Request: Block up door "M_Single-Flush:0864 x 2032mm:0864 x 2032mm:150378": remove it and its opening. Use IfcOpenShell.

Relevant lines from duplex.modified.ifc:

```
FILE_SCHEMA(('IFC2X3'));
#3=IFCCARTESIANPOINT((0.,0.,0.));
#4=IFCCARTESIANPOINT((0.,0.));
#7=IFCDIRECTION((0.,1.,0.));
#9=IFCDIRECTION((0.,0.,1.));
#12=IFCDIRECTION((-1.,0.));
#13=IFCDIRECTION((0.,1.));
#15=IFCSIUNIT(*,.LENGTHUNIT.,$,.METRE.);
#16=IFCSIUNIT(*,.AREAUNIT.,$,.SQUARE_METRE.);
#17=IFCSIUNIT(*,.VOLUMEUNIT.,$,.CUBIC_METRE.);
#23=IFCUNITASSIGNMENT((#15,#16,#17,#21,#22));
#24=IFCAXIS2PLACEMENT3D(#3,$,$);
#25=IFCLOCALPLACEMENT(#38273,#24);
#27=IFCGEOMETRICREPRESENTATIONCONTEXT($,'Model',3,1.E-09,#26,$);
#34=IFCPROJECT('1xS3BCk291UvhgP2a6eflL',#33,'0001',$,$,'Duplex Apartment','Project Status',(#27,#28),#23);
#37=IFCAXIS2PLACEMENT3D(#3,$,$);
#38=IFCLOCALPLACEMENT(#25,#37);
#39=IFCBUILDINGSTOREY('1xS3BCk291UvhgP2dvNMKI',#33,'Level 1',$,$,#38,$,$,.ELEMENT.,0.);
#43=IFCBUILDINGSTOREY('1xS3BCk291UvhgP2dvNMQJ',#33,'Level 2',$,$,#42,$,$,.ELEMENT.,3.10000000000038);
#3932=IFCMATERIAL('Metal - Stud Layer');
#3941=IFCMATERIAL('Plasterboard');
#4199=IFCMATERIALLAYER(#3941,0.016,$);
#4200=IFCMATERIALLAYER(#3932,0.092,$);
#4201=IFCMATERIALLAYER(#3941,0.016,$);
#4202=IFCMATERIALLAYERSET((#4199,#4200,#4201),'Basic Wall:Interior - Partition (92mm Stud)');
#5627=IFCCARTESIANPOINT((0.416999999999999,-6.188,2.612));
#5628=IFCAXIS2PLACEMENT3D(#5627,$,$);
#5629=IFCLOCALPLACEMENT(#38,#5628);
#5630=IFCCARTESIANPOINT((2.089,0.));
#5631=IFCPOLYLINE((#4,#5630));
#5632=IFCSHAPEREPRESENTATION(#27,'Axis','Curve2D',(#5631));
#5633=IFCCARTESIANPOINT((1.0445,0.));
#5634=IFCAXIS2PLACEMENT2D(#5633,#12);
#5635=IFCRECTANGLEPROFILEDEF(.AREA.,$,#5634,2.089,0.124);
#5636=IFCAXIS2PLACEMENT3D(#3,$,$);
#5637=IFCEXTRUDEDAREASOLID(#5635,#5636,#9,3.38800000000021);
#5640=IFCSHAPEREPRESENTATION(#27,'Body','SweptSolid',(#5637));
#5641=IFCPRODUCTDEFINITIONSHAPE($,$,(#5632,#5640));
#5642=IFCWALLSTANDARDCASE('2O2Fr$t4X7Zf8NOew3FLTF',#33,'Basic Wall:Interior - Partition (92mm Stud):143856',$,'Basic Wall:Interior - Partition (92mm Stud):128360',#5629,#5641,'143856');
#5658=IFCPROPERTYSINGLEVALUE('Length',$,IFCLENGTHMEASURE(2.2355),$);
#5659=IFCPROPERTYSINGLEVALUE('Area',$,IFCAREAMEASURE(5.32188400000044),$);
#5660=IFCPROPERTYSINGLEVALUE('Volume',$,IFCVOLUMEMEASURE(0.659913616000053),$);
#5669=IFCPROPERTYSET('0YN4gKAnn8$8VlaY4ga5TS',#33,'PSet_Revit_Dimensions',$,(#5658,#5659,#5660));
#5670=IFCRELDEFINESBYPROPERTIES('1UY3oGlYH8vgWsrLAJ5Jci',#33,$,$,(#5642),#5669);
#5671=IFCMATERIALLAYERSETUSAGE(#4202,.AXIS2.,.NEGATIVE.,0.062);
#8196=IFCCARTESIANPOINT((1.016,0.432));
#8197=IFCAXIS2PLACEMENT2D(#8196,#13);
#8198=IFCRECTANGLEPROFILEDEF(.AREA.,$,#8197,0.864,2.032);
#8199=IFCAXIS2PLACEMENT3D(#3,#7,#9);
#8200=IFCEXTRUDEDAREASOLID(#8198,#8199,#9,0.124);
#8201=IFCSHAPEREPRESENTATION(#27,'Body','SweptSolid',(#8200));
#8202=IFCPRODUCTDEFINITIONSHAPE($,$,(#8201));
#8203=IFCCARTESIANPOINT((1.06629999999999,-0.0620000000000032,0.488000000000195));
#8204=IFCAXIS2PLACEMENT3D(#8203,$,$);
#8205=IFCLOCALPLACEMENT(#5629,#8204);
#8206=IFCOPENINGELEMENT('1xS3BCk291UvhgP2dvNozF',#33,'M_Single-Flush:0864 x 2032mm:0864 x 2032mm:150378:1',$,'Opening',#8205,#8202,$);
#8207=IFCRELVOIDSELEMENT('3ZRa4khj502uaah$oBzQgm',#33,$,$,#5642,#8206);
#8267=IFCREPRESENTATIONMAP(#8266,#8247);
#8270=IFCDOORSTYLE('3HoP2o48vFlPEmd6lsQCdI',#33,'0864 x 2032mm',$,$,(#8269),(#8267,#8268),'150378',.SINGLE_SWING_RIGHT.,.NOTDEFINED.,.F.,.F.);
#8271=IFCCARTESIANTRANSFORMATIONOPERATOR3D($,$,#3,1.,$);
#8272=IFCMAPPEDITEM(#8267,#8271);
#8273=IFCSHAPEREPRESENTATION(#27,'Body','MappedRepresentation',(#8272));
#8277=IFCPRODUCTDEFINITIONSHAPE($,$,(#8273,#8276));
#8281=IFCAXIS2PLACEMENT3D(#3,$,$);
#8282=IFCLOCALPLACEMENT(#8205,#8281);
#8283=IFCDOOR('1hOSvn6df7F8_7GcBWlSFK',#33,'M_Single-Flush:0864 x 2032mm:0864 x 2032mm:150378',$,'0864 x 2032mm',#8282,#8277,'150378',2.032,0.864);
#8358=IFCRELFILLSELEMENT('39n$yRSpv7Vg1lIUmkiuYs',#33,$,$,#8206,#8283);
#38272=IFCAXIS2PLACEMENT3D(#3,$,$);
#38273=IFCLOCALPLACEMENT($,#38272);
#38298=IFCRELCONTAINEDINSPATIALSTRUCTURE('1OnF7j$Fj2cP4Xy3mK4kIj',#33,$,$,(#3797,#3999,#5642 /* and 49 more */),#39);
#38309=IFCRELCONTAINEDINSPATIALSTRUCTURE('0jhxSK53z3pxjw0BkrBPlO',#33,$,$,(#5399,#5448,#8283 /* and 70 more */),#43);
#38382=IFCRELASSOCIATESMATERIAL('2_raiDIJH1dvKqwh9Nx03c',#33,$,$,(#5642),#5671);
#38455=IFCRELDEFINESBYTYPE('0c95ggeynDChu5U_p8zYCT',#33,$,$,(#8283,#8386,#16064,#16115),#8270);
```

```python
import ifcopenshell
import ifcopenshell.api.feature
import ifcopenshell.api.pset
import ifcopenshell.api.root
import ifcopenshell.geom
import ifcopenshell.util.element
import ifcopenshell.util.shape
import ifcopenshell.util.unit

model = ifcopenshell.open("duplex.modified.ifc")
area_scale = ifcopenshell.util.unit.calculate_unit_scale(model, "AREAUNIT")
volume_scale = ifcopenshell.util.unit.calculate_unit_scale(model, "VOLUMEUNIT")
settings = ifcopenshell.geom.settings()


def volume(element):
    """Net volume in cubic metres, openings subtracted."""
    shape = ifcopenshell.geom.create_shape(settings, element)
    return ifcopenshell.util.shape.get_volume(shape.geometry)


door = model.by_guid("1hOSvn6df7F8_7GcBWlSFK")
opening = door.FillsVoids[0].RelatingOpeningElement
wall = opening.VoidsElements[0].RelatingBuildingElement
before = volume(wall)

ifcopenshell.api.root.remove_product(model, product=door)
ifcopenshell.api.feature.remove_feature(model, feature=opening)

after = volume(wall)
thickness = 0.124  # wall thickness in metres

# Update the wall's stored quantities.
pset = model.by_id(ifcopenshell.util.element.get_pset(wall, "PSet_Revit_Dimensions", should_inherit=False)["id"])
ifcopenshell.api.pset.edit_pset(model, pset=pset, properties={
    "Area": model.create_entity("IfcAreaMeasure", after / thickness / area_scale),
    "Volume": model.create_entity("IfcVolumeMeasure", after / volume_scale),
})

print(f"wall volume {before:.3f} -> {after:.3f} m3")

model.write("duplex.modified_updated.ifc")
```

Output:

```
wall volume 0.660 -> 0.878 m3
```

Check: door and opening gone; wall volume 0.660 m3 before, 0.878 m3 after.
